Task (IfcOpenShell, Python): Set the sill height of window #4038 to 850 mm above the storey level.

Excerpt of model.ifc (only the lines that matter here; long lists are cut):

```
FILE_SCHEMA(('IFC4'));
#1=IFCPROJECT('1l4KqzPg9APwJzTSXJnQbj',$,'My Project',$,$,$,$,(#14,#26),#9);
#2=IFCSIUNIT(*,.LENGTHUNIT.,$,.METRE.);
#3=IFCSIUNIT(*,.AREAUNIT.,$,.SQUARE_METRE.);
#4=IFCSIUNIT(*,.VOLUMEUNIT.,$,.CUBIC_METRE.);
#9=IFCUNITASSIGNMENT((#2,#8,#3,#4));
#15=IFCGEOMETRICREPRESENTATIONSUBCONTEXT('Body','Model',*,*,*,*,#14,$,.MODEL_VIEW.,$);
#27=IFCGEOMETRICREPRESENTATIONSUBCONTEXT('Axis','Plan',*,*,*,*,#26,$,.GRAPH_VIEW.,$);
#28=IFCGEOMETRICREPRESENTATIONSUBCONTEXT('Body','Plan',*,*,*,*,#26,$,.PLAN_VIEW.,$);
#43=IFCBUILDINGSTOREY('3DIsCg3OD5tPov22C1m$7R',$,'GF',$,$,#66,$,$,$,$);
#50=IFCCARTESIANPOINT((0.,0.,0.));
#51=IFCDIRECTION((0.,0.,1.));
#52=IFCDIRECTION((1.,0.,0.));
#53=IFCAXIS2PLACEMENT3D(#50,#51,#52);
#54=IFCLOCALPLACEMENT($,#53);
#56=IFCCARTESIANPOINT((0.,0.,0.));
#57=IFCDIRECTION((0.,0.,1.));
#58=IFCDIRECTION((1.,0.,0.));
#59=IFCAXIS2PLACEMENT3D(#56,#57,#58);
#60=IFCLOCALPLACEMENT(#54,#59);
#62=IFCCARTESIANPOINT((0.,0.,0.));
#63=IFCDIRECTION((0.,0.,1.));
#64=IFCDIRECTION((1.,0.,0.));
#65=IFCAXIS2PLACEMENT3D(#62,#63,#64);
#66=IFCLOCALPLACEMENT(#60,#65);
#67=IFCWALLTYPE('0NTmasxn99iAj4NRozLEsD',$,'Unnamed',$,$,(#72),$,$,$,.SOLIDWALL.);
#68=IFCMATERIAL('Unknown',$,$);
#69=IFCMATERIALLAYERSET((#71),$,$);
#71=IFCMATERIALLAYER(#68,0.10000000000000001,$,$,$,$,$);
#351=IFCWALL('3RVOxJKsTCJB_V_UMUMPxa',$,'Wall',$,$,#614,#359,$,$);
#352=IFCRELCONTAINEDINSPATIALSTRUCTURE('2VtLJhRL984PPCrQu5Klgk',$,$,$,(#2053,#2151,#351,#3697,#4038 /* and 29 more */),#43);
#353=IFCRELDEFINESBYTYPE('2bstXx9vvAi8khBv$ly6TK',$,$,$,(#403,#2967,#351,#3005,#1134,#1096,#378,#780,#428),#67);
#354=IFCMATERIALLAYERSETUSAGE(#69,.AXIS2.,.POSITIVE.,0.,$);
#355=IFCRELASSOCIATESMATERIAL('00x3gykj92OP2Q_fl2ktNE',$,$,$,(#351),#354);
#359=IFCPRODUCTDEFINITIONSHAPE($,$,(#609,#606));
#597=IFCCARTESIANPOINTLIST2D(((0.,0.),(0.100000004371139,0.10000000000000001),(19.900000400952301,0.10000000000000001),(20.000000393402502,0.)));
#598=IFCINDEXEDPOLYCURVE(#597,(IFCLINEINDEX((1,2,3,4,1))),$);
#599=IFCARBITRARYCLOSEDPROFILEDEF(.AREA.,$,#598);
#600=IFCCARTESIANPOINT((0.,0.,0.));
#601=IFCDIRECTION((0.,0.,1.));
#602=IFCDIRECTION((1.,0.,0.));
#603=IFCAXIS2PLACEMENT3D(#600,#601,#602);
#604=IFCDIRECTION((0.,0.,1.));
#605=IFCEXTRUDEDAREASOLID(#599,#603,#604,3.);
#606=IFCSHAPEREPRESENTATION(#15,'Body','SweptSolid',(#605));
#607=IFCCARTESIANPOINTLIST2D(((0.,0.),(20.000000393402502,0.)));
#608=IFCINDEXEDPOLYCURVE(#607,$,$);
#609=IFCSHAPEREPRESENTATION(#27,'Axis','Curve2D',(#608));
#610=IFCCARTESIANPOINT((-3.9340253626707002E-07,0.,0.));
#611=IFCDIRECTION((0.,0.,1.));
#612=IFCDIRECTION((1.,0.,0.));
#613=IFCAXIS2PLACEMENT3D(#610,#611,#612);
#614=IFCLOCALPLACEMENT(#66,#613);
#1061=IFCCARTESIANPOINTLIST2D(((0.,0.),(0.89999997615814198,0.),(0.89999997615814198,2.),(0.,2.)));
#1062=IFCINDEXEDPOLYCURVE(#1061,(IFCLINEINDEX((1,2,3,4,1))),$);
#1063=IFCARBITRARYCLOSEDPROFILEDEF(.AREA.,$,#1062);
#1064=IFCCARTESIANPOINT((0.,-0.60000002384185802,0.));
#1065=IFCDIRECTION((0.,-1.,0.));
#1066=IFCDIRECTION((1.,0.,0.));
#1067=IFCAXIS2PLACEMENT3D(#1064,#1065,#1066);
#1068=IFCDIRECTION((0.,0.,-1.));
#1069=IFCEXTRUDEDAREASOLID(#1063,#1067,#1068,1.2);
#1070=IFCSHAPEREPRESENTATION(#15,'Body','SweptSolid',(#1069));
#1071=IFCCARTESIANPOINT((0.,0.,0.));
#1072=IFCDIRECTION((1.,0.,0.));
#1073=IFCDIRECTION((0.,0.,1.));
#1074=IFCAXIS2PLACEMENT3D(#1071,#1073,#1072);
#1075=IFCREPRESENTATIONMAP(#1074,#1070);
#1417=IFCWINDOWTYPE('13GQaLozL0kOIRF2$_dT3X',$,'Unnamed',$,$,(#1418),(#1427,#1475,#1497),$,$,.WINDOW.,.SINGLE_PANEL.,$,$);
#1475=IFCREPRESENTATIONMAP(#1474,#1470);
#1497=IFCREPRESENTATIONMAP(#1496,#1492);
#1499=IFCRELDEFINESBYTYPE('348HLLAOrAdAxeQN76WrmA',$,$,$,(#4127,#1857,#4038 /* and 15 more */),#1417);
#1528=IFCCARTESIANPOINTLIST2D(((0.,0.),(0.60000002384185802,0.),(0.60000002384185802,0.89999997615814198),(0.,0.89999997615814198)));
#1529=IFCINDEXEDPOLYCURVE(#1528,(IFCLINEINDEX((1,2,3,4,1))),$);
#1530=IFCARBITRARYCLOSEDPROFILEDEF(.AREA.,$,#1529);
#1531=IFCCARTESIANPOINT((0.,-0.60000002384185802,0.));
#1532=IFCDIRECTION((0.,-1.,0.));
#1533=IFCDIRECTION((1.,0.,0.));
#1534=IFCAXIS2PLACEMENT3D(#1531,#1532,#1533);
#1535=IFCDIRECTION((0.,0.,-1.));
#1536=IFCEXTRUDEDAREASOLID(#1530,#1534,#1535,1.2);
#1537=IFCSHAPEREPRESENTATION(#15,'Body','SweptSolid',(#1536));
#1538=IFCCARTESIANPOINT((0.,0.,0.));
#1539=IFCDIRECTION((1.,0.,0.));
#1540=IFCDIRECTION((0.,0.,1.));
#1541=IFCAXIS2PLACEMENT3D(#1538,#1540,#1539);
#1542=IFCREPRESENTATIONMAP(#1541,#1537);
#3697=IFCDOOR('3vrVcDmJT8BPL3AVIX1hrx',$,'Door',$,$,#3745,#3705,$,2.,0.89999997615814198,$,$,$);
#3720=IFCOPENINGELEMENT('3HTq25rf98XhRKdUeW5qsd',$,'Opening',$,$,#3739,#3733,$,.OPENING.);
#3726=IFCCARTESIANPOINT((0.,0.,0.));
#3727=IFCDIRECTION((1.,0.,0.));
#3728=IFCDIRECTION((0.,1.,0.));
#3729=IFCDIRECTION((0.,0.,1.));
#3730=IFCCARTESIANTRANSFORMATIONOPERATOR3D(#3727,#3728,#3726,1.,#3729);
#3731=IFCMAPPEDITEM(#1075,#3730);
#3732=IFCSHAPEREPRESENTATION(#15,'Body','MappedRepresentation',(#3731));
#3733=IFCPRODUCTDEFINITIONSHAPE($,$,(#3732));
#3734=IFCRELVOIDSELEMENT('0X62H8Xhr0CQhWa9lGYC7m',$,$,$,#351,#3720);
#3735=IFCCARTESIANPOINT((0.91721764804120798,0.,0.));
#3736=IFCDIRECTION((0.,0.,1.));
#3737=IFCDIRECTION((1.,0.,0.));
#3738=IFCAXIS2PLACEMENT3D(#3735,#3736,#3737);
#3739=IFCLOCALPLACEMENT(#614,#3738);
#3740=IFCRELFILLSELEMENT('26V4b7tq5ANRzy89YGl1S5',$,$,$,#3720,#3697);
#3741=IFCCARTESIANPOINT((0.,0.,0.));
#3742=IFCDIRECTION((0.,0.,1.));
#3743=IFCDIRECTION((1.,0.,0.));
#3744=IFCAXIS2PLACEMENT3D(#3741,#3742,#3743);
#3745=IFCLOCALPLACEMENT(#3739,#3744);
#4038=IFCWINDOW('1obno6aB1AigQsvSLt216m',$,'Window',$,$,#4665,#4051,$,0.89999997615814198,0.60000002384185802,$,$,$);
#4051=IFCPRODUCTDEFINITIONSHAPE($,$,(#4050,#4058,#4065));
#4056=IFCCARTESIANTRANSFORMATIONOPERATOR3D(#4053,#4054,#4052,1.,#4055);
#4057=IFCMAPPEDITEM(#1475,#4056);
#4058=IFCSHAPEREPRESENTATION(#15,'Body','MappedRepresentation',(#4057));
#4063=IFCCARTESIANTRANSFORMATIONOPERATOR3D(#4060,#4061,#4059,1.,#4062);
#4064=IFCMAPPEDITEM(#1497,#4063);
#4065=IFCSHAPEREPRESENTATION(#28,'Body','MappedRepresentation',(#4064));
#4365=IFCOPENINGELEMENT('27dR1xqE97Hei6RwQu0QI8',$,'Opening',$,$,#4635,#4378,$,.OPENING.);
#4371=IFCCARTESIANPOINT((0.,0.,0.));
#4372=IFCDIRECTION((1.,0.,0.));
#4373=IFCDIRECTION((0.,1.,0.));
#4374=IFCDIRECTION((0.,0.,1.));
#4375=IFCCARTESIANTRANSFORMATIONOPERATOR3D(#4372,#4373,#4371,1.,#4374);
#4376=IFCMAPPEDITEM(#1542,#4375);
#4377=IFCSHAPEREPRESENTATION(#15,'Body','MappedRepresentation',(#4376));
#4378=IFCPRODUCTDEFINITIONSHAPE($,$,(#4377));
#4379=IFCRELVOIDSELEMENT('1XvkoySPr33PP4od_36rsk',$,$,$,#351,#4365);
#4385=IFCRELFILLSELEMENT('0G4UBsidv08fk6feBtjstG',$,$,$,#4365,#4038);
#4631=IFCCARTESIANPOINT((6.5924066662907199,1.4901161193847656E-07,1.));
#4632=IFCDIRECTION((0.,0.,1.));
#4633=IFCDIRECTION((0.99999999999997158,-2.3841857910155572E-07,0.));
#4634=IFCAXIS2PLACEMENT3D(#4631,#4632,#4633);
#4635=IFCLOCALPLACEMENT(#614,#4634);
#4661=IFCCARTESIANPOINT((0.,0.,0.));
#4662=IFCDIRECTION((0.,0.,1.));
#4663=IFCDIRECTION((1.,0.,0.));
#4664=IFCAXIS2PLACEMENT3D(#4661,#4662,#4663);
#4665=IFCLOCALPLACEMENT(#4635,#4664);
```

```python
import numpy as np
import ifcopenshell
import ifcopenshell.api.geometry
import ifcopenshell.geom
import ifcopenshell.util.element
import ifcopenshell.util.placement
import ifcopenshell.util.shape
import ifcopenshell.util.unit

model = ifcopenshell.open("model.ifc")
unit_scale = ifcopenshell.util.unit.calculate_unit_scale(model)

window = model.by_guid("1obno6aB1AigQsvSLt216m")
opening = window.FillsVoids[0].RelatingOpeningElement
storey = ifcopenshell.util.element.get_container(window, ifc_class="IfcBuildingStorey")
level = ifcopenshell.util.placement.get_local_placement(storey.ObjectPlacement)[2, 3]

# The opening's origin need not be at the sill, so measure its lowest point.
shape = ifcopenshell.geom.create_shape(ifcopenshell.geom.settings(), opening)
bottom = ifcopenshell.util.shape.get_shape_bottom_elevation(shape, shape.geometry) / unit_scale
dz = level + 0.85 / unit_scale - bottom

shift = np.array([0.0, 0.0, dz])
# The window is placed relative to its opening, so it follows when the opening moves.
matrix = ifcopenshell.util.placement.get_local_placement(opening.ObjectPlacement)
matrix[:3, 3] += shift
ifcopenshell.api.geometry.edit_object_placement(
    model, product=opening, matrix=matrix, is_si=False, should_transform_children=True
)

print(f"moved by {dz * unit_scale:+.3f} m")

model.write("model_v2.ifc")
```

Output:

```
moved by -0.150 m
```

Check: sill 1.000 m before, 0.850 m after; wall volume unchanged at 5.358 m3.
